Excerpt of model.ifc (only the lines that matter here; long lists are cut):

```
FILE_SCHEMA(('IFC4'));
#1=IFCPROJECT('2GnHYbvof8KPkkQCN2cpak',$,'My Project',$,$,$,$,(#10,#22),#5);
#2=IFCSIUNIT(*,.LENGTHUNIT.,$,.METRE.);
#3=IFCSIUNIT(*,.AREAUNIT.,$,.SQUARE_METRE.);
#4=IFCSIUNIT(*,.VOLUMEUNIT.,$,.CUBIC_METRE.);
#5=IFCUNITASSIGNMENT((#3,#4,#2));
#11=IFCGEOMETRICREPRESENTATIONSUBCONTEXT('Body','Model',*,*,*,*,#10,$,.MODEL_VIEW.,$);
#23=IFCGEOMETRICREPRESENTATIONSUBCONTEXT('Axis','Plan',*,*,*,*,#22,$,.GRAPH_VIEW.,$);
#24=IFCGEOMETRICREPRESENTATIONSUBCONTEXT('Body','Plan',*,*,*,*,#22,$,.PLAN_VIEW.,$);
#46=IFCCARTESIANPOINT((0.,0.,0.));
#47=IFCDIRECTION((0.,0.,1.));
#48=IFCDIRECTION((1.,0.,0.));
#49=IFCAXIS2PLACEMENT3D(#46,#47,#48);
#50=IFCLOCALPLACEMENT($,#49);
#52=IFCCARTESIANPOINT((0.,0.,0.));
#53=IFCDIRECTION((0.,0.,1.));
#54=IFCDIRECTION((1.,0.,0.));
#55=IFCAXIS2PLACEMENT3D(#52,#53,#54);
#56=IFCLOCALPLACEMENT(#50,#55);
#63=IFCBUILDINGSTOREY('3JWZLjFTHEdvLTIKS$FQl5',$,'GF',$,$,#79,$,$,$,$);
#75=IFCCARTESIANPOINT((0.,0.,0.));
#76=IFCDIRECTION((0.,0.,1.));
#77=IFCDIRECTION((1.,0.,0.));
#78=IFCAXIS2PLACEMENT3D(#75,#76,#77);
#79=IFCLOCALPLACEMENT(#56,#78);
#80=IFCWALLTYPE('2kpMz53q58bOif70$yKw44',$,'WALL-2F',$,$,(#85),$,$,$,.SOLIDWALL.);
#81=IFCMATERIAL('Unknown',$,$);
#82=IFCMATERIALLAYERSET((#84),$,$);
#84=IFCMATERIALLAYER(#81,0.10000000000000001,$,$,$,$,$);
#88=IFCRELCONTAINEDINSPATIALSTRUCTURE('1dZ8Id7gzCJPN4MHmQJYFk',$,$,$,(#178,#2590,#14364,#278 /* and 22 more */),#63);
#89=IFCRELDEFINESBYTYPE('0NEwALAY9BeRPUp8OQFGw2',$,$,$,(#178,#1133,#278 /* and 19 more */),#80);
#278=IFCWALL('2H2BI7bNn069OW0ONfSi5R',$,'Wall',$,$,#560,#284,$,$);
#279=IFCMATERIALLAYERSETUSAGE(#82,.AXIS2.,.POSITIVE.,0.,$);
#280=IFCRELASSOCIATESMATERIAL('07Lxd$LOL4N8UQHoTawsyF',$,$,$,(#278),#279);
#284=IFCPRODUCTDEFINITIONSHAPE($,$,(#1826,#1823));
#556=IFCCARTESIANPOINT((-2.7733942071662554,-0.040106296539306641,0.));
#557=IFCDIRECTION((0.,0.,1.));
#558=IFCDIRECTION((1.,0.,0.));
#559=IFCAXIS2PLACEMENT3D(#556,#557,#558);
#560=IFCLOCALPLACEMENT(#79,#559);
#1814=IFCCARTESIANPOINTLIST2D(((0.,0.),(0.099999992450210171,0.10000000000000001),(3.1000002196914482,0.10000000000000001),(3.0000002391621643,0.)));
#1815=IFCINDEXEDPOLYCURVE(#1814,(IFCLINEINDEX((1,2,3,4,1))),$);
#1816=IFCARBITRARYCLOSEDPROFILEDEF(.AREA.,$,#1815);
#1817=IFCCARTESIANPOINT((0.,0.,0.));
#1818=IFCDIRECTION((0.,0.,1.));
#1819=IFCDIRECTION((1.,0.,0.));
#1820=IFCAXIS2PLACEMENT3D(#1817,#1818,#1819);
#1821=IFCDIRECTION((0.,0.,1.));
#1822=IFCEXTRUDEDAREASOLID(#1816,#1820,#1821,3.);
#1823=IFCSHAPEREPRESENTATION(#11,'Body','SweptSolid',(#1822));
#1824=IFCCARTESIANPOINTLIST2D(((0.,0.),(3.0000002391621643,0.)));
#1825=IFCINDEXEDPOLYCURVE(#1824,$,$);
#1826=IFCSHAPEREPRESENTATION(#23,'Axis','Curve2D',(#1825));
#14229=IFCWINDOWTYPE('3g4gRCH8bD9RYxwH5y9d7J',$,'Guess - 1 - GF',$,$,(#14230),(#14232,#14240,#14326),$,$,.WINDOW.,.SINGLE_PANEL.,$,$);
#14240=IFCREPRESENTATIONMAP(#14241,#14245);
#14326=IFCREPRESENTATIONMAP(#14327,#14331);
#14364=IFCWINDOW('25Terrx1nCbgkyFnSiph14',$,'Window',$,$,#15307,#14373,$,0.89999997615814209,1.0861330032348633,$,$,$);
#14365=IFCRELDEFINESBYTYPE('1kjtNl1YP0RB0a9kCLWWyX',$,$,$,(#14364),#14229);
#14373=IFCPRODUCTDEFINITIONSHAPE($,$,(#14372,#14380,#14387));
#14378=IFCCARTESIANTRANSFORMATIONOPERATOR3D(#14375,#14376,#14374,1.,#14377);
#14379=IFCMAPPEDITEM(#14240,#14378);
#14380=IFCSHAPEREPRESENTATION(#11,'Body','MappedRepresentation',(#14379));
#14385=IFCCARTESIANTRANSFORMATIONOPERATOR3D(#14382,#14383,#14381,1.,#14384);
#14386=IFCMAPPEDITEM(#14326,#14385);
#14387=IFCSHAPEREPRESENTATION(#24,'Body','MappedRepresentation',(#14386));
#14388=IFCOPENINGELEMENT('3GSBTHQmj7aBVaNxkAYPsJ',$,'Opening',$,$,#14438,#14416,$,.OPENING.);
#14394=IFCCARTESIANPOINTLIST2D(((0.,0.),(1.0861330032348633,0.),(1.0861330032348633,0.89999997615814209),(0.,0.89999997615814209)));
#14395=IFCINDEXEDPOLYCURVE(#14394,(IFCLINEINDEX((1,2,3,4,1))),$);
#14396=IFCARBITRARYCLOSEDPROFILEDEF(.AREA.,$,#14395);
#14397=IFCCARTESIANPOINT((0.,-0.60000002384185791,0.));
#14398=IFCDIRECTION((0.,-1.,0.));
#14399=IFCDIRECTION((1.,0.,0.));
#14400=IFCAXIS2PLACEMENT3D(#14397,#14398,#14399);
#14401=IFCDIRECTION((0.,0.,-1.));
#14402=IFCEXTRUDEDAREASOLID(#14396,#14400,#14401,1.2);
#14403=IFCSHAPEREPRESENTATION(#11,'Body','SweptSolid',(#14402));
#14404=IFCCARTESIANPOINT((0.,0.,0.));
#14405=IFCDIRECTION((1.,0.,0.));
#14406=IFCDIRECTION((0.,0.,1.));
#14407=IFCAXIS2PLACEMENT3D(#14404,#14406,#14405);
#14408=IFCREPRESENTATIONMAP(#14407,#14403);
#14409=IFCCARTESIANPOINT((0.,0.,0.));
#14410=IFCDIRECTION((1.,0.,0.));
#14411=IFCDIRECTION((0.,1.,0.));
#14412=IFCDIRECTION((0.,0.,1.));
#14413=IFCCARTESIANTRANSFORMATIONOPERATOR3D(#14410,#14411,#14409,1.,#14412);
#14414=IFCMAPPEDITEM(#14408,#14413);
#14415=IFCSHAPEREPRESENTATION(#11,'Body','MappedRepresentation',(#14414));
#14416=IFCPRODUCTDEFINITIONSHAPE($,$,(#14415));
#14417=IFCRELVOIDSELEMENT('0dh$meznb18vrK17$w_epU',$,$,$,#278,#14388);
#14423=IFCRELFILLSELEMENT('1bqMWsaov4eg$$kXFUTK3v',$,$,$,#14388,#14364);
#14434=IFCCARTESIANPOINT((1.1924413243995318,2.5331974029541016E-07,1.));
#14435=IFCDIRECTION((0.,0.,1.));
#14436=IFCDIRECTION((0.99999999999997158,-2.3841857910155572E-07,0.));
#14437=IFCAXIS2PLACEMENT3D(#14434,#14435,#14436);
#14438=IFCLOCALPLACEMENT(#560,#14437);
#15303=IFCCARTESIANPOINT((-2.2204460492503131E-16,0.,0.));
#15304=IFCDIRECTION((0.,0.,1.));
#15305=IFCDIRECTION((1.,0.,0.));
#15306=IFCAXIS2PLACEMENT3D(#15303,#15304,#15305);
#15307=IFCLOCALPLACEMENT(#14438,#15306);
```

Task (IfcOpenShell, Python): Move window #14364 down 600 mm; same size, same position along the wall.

```python
import numpy as np
import ifcopenshell
import ifcopenshell.api.geometry
import ifcopenshell.util.placement
import ifcopenshell.util.unit

model = ifcopenshell.open("model.ifc")
unit_scale = ifcopenshell.util.unit.calculate_unit_scale(model)

window = model.by_guid("25Terrx1nCbgkyFnSiph14")
opening = window.FillsVoids[0].RelatingOpeningElement
dz = -0.6

shift = np.array([0.0, 0.0, dz])
# The window is placed relative to its opening, so it follows when the opening moves.
matrix = ifcopenshell.util.placement.get_local_placement(opening.ObjectPlacement)
matrix[:3, 3] += shift
ifcopenshell.api.geometry.edit_object_placement(
    model, product=opening, matrix=matrix, is_si=False, should_transform_children=True
)

print(f"moved by {dz * unit_scale:+.3f} m")

model.write("model-out.ifc")
```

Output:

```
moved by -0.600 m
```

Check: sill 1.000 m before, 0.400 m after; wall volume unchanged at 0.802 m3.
